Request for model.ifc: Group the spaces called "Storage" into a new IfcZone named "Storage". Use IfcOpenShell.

First a look at what the model holds.

```python
import ifcopenshell

model = ifcopenshell.open("model.ifc")
print(model.schema)
seen = {}
for space in model.by_type("IfcSpace"):
    seen[space.LongName] = seen.get(space.LongName, 0) + 1
for name, count in sorted(seen.items(), key=str):
    print(count, "x", name)
print("zones:", [z.Name for z in model.by_type("IfcZone")][:20])
```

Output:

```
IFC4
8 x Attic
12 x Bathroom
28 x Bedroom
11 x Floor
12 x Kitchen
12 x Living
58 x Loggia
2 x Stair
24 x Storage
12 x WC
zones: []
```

```python
import ifcopenshell
import ifcopenshell.api.group
import ifcopenshell.api.root

model = ifcopenshell.open("model.ifc")

names = {"Storage"}
spaces = [s for s in model.by_type("IfcSpace") if s.LongName in names]

zone = ifcopenshell.api.root.create_entity(model, ifc_class="IfcZone", name="Storage")
ifcopenshell.api.group.assign_group(model, products=spaces, group=zone)
print(len(spaces), "spaces in", zone.Name)

model.write("model_updated.ifc")
```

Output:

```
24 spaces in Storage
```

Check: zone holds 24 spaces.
